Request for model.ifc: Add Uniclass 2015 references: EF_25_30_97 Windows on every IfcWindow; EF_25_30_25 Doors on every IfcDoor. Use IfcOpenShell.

First a look at what the model holds.

```python
import ifcopenshell

model = ifcopenshell.open("model.ifc")
print(model.schema)
print("classifications:", [c.Name for c in model.by_type("IfcClassification")])
for ifc_class in ("IfcDoor", "IfcRoof", "IfcStair", "IfcWall", "IfcWindow"):
    print(ifc_class, len(model.by_type(ifc_class)))
```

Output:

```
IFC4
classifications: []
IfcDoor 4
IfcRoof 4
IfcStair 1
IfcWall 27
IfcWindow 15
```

```python
import ifcopenshell
import ifcopenshell.api.classification

model = ifcopenshell.open("model.ifc")

system = ifcopenshell.api.classification.add_classification(model, classification="Uniclass 2015")

codes = {
    "IfcWindow": ("EF_25_30_97", "Windows"),
    "IfcDoor": ("EF_25_30_25", "Doors"),
}
for ifc_class, (code, name) in codes.items():
    products = model.by_type(ifc_class)
    ifcopenshell.api.classification.add_reference(
        model, products=products, classification=system, identification=code, name=name
    )
    print(code, len(products))

model.write("model_edited.ifc")
```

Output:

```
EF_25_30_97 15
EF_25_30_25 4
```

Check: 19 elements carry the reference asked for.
